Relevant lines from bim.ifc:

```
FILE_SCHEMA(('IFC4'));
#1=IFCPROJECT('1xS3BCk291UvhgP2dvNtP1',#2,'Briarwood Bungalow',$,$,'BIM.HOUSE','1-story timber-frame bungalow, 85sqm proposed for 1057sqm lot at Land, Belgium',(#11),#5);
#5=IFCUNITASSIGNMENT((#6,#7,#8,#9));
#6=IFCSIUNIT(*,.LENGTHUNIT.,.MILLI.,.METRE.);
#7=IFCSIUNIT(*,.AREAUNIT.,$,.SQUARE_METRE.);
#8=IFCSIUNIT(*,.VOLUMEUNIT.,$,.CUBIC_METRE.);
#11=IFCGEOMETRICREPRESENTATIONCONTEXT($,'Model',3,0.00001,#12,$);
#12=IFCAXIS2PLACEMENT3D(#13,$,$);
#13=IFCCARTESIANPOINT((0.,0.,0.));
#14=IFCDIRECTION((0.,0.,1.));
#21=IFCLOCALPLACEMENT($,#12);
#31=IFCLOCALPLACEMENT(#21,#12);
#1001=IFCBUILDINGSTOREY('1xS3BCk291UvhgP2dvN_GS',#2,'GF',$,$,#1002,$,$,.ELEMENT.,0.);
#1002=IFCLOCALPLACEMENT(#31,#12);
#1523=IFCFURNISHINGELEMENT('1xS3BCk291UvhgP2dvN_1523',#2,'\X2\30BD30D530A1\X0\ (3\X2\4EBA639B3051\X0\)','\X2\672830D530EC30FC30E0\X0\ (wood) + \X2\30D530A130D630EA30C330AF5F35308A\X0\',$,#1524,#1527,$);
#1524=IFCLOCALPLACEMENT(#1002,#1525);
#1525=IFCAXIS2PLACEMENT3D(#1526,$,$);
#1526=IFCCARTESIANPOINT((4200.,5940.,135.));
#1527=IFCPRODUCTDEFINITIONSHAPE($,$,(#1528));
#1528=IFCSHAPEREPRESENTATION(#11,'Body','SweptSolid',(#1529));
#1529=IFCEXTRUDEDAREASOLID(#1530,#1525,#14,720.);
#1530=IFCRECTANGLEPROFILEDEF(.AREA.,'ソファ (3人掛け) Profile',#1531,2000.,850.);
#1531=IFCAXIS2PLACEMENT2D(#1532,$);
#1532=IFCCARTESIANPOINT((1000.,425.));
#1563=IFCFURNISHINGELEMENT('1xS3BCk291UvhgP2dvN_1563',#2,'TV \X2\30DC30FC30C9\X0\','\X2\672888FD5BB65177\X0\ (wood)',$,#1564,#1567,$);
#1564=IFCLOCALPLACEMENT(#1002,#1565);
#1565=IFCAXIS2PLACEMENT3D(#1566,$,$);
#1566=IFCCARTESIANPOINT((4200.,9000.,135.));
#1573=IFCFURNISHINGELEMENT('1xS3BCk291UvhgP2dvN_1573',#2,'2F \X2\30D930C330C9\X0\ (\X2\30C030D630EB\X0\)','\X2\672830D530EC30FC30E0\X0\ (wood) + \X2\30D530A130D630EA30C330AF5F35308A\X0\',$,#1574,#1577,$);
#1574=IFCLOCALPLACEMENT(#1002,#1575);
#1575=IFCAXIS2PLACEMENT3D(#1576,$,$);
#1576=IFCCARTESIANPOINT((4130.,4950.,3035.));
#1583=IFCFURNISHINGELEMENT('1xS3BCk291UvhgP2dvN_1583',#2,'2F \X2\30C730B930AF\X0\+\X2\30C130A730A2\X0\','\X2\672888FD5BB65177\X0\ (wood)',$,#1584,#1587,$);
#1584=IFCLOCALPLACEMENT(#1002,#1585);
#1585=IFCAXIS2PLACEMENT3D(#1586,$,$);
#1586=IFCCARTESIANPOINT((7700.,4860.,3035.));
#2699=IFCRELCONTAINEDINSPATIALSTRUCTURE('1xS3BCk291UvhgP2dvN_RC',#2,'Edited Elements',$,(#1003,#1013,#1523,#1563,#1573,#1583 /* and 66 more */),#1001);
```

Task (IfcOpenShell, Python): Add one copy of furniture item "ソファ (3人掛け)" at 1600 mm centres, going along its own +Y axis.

```python
import ifcopenshell
import ifcopenshell.api.geometry
import ifcopenshell.api.root
import ifcopenshell.util.element
import ifcopenshell.util.placement
import ifcopenshell.util.unit

model = ifcopenshell.open("bim.ifc")
unit_scale = ifcopenshell.util.unit.calculate_unit_scale(model)


def reuse_history(source, copy):
    """copy_class also copies each property set's owner history, people and application; keep the originals."""
    for rel in copy.IsDefinedBy:
        if rel.is_a("IfcRelDefinesByProperties") and (history := rel.RelatingPropertyDefinition.OwnerHistory):
            rel.RelatingPropertyDefinition.OwnerHistory = source.OwnerHistory
            ifcopenshell.util.element.remove_deep2(model, history)


source = model.by_guid("1xS3BCk291UvhgP2dvN_1523")
base = ifcopenshell.util.placement.get_local_placement(source.ObjectPlacement)
step = base[:3, 1] * 1.6 / unit_scale

for i in range(1, 2):
    copy = ifcopenshell.api.root.copy_class(model, product=source)
    copy.Representation = ifcopenshell.util.element.copy_deep(
        model, source.Representation, exclude=["IfcGeometricRepresentationContext", "IfcRepresentationMap"]
    )
    reuse_history(source, copy)
    matrix = base.copy()
    matrix[:3, 3] += i * step
    print("added at", matrix[:3, 3].round(3) + 0.0)
    ifcopenshell.api.geometry.edit_object_placement(model, product=copy, matrix=matrix, is_si=False)

model.write("bim_updated.ifc")
```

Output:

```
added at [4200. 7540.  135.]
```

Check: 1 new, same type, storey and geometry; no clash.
